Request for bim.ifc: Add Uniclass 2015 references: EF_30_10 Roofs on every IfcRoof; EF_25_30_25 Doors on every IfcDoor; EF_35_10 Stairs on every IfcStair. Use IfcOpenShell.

First a look at what the model holds.

```python
import ifcopenshell

model = ifcopenshell.open("bim.ifc")
print(model.schema)
print("classifications:", [c.Name for c in model.by_type("IfcClassification")])
for ifc_class in ("IfcDoor", "IfcRoof", "IfcStair", "IfcWall", "IfcWindow"):
    print(ifc_class, len(model.by_type(ifc_class)))
```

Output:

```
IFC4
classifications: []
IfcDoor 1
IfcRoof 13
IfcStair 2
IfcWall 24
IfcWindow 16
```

```python
import ifcopenshell
import ifcopenshell.api.classification

model = ifcopenshell.open("bim.ifc")

system = ifcopenshell.api.classification.add_classification(model, classification="Uniclass 2015")

codes = {
    "IfcRoof": ("EF_30_10", "Roofs"),
    "IfcDoor": ("EF_25_30_25", "Doors"),
    "IfcStair": ("EF_35_10", "Stairs"),
}
for ifc_class, (code, name) in codes.items():
    products = model.by_type(ifc_class)
    ifcopenshell.api.classification.add_reference(
        model, products=products, classification=system, identification=code, name=name
    )
    print(code, len(products))

model.write("bim_v2.ifc")
```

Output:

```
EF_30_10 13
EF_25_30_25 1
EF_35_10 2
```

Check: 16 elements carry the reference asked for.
